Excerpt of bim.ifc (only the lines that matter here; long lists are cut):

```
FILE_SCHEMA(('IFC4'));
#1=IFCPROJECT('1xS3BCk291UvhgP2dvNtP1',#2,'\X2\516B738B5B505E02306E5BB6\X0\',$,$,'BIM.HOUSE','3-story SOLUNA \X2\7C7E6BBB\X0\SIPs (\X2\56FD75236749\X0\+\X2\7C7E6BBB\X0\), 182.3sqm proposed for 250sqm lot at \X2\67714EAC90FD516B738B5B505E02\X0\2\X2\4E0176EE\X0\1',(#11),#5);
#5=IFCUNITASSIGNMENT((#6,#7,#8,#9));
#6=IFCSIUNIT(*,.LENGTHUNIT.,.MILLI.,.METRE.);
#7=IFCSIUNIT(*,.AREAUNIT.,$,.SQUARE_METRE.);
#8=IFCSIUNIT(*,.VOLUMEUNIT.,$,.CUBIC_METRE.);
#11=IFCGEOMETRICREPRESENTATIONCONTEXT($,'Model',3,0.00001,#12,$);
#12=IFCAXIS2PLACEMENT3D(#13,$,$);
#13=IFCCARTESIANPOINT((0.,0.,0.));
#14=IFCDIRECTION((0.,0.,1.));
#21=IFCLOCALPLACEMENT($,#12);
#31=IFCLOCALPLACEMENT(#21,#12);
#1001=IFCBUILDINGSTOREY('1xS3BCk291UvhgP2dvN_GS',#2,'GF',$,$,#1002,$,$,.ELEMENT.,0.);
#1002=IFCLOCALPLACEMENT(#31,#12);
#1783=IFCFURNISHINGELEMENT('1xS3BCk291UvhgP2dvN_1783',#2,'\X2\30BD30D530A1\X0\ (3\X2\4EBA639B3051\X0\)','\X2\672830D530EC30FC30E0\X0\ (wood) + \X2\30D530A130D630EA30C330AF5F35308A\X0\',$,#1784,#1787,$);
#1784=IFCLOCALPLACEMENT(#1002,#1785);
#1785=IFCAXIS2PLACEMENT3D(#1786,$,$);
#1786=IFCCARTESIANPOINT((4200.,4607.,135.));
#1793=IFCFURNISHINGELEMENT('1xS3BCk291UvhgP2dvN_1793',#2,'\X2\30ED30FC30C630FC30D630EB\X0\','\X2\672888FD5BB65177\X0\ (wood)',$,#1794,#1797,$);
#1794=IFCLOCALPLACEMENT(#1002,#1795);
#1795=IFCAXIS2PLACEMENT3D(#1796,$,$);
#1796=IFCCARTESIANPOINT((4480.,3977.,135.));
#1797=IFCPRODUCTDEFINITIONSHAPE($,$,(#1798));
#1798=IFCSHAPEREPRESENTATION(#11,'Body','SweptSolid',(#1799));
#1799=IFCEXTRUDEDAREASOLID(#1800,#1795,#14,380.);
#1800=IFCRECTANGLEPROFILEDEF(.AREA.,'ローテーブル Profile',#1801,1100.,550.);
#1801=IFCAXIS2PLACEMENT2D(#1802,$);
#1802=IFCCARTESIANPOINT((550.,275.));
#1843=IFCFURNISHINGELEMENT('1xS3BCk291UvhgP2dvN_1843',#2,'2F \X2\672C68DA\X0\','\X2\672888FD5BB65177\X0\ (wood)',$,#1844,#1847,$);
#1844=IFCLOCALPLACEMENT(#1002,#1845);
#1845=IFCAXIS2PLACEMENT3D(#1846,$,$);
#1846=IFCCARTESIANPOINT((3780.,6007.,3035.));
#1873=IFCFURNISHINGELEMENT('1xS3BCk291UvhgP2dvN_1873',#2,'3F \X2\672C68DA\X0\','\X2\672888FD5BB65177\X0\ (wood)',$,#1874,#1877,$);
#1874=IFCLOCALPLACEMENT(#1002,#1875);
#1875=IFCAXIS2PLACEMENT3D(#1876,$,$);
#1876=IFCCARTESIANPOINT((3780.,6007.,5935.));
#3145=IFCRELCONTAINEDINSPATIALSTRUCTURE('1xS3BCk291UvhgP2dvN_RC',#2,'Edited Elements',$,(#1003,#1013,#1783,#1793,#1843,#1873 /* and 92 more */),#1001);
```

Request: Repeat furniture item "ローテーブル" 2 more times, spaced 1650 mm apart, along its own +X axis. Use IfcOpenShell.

```python
import ifcopenshell
import ifcopenshell.api.geometry
import ifcopenshell.api.root
import ifcopenshell.util.element
import ifcopenshell.util.placement
import ifcopenshell.util.unit

model = ifcopenshell.open("bim.ifc")
unit_scale = ifcopenshell.util.unit.calculate_unit_scale(model)


def reuse_history(source, copy):
    """copy_class also copies each property set's owner history, people and application; keep the originals."""
    for rel in copy.IsDefinedBy:
        if rel.is_a("IfcRelDefinesByProperties") and (history := rel.RelatingPropertyDefinition.OwnerHistory):
            rel.RelatingPropertyDefinition.OwnerHistory = source.OwnerHistory
            ifcopenshell.util.element.remove_deep2(model, history)


source = model.by_guid("1xS3BCk291UvhgP2dvN_1793")
base = ifcopenshell.util.placement.get_local_placement(source.ObjectPlacement)
step = base[:3, 0] * 1.65 / unit_scale

for i in range(1, 3):
    copy = ifcopenshell.api.root.copy_class(model, product=source)
    copy.Representation = ifcopenshell.util.element.copy_deep(
        model, source.Representation, exclude=["IfcGeometricRepresentationContext", "IfcRepresentationMap"]
    )
    reuse_history(source, copy)
    matrix = base.copy()
    matrix[:3, 3] += i * step
    print("added at", matrix[:3, 3].round(3) + 0.0)
    ifcopenshell.api.geometry.edit_object_placement(model, product=copy, matrix=matrix, is_si=False)

model.write("bim-out.ifc")
```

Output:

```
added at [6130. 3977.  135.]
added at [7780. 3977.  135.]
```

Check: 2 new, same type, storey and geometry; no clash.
